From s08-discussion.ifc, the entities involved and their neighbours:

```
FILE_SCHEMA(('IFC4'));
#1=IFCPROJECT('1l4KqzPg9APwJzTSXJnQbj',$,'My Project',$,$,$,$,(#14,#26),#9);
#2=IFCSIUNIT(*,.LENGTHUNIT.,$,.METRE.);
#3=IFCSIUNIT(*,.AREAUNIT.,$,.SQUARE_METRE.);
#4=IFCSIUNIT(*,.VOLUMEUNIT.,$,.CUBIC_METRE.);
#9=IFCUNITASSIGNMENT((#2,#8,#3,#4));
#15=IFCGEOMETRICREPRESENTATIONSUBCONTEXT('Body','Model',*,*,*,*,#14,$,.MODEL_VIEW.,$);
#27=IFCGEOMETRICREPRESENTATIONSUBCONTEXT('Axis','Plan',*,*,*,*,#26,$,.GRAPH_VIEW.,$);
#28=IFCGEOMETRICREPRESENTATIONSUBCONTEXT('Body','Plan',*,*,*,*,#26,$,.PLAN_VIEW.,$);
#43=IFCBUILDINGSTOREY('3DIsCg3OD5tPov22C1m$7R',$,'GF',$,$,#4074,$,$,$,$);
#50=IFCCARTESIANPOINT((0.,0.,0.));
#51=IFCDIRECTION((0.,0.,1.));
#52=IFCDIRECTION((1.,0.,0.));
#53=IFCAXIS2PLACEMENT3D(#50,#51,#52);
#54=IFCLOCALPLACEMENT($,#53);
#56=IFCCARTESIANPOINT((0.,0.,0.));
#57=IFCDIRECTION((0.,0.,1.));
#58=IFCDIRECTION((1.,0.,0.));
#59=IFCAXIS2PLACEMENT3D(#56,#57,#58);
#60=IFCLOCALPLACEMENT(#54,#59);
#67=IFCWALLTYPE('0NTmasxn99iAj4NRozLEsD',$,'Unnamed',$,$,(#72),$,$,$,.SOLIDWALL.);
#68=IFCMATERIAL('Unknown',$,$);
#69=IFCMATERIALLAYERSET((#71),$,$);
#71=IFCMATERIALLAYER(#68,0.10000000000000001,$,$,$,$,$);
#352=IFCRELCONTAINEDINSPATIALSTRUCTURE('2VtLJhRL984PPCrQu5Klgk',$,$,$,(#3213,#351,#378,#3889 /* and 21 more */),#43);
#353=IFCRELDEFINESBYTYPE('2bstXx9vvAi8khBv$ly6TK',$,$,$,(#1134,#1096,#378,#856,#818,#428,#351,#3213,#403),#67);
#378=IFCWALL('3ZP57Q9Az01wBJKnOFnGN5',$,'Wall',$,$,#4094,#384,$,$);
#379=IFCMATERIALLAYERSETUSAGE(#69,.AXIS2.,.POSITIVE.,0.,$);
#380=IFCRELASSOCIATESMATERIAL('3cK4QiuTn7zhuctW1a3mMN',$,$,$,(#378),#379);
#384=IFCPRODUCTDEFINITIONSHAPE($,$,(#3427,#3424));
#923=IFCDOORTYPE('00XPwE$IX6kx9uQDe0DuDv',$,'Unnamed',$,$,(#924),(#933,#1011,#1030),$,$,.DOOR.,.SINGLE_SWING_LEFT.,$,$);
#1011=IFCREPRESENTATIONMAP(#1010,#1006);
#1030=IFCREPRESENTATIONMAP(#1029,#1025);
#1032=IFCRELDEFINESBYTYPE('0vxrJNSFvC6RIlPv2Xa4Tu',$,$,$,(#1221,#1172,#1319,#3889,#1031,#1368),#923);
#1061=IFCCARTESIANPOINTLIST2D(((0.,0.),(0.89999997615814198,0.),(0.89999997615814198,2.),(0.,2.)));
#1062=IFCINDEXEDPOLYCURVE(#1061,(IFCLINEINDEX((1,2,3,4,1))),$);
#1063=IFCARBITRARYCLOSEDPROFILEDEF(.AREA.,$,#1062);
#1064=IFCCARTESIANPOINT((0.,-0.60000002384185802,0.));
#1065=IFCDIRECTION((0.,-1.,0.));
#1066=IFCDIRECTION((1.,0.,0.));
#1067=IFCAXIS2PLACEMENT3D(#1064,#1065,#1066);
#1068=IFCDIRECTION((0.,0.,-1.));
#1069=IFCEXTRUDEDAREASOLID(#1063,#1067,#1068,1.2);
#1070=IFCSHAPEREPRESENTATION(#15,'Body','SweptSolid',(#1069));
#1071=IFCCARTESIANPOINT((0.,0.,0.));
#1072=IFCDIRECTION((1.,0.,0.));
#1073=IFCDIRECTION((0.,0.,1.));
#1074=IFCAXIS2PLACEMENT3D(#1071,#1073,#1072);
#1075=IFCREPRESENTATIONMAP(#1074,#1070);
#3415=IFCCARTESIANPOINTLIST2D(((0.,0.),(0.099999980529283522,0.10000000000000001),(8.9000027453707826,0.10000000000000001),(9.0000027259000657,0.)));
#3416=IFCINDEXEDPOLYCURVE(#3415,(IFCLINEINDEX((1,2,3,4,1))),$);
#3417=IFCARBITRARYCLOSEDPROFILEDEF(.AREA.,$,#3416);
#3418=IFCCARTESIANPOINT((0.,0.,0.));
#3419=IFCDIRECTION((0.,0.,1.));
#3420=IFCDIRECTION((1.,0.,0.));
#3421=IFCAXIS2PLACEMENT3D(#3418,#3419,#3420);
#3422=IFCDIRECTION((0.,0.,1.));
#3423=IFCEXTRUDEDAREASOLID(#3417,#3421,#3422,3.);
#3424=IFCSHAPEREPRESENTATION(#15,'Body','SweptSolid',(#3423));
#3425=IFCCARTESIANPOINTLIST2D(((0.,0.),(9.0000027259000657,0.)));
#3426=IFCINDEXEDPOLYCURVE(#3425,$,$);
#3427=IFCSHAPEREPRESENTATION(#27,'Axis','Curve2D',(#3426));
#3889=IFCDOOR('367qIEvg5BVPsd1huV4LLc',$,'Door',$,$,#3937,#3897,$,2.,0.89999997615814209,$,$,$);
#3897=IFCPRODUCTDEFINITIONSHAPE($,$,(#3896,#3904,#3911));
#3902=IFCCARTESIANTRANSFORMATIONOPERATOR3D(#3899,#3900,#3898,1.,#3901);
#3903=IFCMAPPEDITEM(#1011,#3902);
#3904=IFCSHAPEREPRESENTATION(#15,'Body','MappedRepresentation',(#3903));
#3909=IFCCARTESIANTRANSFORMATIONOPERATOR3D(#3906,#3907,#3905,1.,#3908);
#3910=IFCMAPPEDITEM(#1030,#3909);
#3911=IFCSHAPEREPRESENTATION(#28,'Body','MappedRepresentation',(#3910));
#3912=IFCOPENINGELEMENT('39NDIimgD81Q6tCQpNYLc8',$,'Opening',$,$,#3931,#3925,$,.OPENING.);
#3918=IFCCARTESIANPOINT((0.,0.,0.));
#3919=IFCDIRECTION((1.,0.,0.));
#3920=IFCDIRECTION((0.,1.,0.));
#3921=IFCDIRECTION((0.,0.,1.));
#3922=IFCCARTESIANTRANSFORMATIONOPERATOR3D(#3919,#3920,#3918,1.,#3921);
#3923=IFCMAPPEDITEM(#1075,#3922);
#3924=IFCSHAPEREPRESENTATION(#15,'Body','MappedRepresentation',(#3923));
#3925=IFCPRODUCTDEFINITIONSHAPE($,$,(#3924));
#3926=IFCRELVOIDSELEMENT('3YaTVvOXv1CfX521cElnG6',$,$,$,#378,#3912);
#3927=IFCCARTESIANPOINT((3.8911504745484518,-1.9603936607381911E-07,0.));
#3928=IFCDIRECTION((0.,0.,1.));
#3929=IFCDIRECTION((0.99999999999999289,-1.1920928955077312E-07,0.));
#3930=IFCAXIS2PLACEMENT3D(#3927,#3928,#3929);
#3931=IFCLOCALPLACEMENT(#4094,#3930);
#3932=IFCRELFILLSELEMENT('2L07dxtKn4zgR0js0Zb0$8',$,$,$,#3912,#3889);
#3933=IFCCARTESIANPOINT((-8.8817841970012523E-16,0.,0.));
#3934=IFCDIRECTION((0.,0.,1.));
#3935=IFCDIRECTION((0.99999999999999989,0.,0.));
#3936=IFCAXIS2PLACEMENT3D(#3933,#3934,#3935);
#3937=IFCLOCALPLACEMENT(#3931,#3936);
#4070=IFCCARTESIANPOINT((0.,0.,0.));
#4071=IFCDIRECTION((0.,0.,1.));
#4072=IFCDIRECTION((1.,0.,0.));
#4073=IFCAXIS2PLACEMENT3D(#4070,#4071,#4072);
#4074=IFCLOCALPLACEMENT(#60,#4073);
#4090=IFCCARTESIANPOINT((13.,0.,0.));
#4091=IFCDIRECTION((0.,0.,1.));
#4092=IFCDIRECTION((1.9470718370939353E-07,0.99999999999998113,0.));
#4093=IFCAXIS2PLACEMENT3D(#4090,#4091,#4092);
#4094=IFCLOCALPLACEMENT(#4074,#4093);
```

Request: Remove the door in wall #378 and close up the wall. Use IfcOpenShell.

```python
import ifcopenshell
import ifcopenshell.api.feature
import ifcopenshell.api.root
import ifcopenshell.geom
import ifcopenshell.util.shape

model = ifcopenshell.open("s08-discussion.ifc")
settings = ifcopenshell.geom.settings()


def volume(element):
    """Net volume in cubic metres, openings subtracted."""
    shape = ifcopenshell.geom.create_shape(settings, element)
    return ifcopenshell.util.shape.get_volume(shape.geometry)


door = model.by_guid("367qIEvg5BVPsd1huV4LLc")
opening = door.FillsVoids[0].RelatingOpeningElement
wall = opening.VoidsElements[0].RelatingBuildingElement
before = volume(wall)

ifcopenshell.api.root.remove_product(model, product=door)
ifcopenshell.api.feature.remove_feature(model, feature=opening)

after = volume(wall)

print(f"wall volume {before:.3f} -> {after:.3f} m3")

model.write("s08-discussion_rev.ifc")
```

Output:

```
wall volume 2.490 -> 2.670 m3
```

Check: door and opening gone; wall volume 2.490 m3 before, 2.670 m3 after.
